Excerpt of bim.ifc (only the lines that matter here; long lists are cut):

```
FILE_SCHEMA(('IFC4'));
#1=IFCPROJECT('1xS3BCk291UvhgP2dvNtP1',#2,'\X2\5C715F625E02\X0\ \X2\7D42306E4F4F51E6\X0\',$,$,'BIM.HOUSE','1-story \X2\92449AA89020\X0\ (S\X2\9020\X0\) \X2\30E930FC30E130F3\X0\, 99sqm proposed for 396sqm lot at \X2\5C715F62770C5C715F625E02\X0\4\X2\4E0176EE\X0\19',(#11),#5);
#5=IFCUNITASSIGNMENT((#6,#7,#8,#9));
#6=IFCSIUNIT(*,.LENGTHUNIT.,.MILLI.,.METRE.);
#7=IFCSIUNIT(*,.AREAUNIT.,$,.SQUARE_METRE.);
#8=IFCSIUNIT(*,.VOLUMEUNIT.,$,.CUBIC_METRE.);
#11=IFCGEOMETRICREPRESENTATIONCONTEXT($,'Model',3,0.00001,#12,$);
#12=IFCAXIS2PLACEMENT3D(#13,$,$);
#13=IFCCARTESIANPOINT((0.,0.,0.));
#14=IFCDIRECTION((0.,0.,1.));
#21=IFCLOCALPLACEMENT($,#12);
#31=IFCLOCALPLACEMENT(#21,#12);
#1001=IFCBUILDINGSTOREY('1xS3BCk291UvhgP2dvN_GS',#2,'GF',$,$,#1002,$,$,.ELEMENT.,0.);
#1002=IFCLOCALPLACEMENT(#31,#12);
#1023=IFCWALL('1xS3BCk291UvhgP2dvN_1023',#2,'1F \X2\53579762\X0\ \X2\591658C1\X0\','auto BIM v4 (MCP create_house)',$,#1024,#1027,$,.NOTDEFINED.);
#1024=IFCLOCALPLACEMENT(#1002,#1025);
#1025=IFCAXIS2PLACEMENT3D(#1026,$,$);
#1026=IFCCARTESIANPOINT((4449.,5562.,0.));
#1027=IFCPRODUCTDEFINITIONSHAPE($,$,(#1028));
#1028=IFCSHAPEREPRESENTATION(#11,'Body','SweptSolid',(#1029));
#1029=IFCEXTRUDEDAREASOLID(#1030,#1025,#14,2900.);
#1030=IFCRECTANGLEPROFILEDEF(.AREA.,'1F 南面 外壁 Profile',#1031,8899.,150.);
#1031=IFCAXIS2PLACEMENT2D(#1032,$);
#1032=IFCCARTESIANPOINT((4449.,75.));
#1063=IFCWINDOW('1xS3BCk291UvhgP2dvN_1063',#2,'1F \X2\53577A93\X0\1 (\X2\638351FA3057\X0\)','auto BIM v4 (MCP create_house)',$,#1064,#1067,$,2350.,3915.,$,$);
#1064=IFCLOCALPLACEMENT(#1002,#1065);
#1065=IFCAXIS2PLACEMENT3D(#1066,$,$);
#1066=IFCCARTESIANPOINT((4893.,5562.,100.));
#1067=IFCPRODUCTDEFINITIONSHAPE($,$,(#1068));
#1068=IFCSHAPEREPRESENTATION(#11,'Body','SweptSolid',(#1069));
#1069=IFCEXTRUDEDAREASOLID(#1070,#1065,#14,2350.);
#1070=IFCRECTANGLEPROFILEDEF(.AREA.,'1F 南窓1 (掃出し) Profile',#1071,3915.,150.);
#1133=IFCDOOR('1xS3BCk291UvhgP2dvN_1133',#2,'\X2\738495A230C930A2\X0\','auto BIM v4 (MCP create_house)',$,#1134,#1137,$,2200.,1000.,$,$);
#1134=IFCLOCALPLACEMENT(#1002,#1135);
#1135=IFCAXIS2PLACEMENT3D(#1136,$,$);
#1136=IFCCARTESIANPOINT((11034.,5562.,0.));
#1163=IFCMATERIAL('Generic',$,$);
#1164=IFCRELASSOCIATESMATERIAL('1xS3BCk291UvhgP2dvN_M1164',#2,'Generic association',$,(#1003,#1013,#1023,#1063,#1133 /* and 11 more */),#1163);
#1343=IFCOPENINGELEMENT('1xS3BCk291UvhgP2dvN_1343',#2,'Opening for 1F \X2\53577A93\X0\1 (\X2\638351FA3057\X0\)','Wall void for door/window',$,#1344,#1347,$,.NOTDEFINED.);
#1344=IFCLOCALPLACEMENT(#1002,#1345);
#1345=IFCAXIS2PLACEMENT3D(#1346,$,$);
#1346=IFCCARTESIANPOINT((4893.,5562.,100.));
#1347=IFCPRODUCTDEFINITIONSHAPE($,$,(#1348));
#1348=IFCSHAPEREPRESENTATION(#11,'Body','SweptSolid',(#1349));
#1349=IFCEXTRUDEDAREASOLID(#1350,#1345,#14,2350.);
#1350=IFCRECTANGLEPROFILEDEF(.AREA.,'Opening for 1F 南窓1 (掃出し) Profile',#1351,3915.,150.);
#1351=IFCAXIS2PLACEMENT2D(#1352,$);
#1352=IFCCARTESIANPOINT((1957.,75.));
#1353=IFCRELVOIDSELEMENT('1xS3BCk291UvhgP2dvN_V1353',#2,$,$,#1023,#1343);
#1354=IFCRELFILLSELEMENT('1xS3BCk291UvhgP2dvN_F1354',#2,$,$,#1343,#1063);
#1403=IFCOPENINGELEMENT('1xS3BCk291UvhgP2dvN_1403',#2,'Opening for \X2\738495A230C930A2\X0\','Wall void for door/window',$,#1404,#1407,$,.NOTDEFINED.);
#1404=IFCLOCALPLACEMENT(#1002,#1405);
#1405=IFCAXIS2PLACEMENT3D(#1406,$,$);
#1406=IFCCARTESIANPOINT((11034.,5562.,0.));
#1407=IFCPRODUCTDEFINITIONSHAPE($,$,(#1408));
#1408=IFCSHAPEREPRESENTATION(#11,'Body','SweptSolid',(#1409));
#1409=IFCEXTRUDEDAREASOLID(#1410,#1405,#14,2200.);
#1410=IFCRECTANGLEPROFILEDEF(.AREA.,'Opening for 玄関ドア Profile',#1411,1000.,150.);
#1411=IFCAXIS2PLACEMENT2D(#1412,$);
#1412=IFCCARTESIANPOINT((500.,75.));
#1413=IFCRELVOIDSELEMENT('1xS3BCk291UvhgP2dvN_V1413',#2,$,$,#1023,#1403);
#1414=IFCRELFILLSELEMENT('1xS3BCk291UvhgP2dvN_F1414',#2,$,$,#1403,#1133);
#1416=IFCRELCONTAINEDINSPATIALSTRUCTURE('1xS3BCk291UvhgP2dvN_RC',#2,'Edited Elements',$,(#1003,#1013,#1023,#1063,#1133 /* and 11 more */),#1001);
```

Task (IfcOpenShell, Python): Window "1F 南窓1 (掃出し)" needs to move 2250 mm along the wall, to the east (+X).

```python
import ifcopenshell
import ifcopenshell.api.geometry
import ifcopenshell.util.placement

model = ifcopenshell.open("bim.ifc")

window = model.by_id(1063)
opening = window.FillsVoids[0].RelatingOpeningElement
wall = opening.VoidsElements[0].RelatingBuildingElement

wall_matrix = ifcopenshell.util.placement.get_local_placement(wall.ObjectPlacement)
shift = wall_matrix[:3, 0] * 2250.0
before = ifcopenshell.util.placement.get_local_placement(window.ObjectPlacement)[:3, 3].copy()

# The window is not placed relative to its opening, so move both.
for product in (opening, window):
    matrix = ifcopenshell.util.placement.get_local_placement(product.ObjectPlacement)
    matrix[:3, 3] += shift
    ifcopenshell.api.geometry.edit_object_placement(model, product=product, matrix=matrix, is_si=False)

after = ifcopenshell.util.placement.get_local_placement(window.ObjectPlacement)[:3, 3]
print("window moved by", (after - before).round(3) + 0.0)

model.write("bim_rev.ifc")
```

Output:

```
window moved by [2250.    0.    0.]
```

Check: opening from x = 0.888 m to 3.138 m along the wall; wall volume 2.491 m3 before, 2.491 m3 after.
